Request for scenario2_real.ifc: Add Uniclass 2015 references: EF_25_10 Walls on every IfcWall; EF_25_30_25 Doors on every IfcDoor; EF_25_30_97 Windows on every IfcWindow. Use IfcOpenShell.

First a look at what the model holds.

```python
import ifcopenshell

model = ifcopenshell.open("scenario2_real.ifc")
print(model.schema)
print("classifications:", [c.Name for c in model.by_type("IfcClassification")])
for ifc_class in ("IfcDoor", "IfcRoof", "IfcStair", "IfcWall", "IfcWindow"):
    print(ifc_class, len(model.by_type(ifc_class)))
```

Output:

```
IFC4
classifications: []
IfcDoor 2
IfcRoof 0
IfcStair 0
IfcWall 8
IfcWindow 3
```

```python
import ifcopenshell
import ifcopenshell.api.classification

model = ifcopenshell.open("scenario2_real.ifc")

system = ifcopenshell.api.classification.add_classification(model, classification="Uniclass 2015")

codes = {
    "IfcWall": ("EF_25_10", "Walls"),
    "IfcDoor": ("EF_25_30_25", "Doors"),
    "IfcWindow": ("EF_25_30_97", "Windows"),
}
for ifc_class, (code, name) in codes.items():
    products = model.by_type(ifc_class)
    ifcopenshell.api.classification.add_reference(
        model, products=products, classification=system, identification=code, name=name
    )
    print(code, len(products))

model.write("scenario2_real_updated.ifc")
```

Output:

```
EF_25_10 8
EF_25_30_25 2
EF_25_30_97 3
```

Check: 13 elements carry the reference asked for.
